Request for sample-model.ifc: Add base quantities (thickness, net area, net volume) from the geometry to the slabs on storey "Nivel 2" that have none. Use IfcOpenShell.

First a look at what the model holds.

```python
import ifcopenshell
import ifcopenshell.util.element
import ifcopenshell.util.unit

model = ifcopenshell.open("sample-model.ifc")
print(model.schema)
for unit_type in ("LENGTHUNIT", "AREAUNIT", "VOLUMEUNIT"):
    print(unit_type, ifcopenshell.util.unit.calculate_unit_scale(model, unit_type))
storey = next(s for s in model.by_type("IfcBuildingStorey") if s.Name == "Nivel 2")
slabs = [e for e in ifcopenshell.util.element.get_decomposition(storey) if e.is_a("IfcSlab")]
for e in sorted(slabs, key=lambda e: e.id()):
    print(e.id(), e.is_a(), e.Name, list(ifcopenshell.util.element.get_psets(e, qtos_only=True)), sep=" | ")
```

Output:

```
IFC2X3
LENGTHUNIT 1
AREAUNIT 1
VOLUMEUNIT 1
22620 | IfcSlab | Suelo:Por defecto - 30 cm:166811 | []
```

```python
import ifcopenshell
import ifcopenshell.api.pset
import ifcopenshell.geom
import ifcopenshell.util.element
import ifcopenshell.util.shape
import ifcopenshell.util.unit

model = ifcopenshell.open("sample-model.ifc")
unit_scale = ifcopenshell.util.unit.calculate_unit_scale(model)
area_scale = ifcopenshell.util.unit.calculate_unit_scale(model, "AREAUNIT")
volume_scale = ifcopenshell.util.unit.calculate_unit_scale(model, "VOLUMEUNIT")
settings = ifcopenshell.geom.settings()

storey = next(s for s in model.by_type("IfcBuildingStorey") if s.Name == "Nivel 2")
slabs = [e for e in ifcopenshell.util.element.get_decomposition(storey) if e.is_a("IfcSlab")]

for e in sorted(slabs, key=lambda e: e.id()):
    if ifcopenshell.util.element.get_psets(e, qtos_only=True, should_inherit=False):
        continue
    # Geometry comes back in metres, in the element's own axes.
    shape = ifcopenshell.geom.create_shape(settings, e)
    values = {
        "Width": ifcopenshell.util.shape.get_z(shape.geometry) / unit_scale,
        "NetArea": ifcopenshell.util.shape.get_footprint_area(shape.geometry) / area_scale,
        "NetVolume": ifcopenshell.util.shape.get_volume(shape.geometry) / volume_scale,
    }
    qto = ifcopenshell.api.pset.add_qto(model, product=e, name="BaseQuantities")
    ifcopenshell.api.pset.edit_qto(model, qto=qto, properties=values)
    print(e.id(), {k: round(v, 3) for k, v in values.items()})

model.write("sample-model_edited.ifc")
```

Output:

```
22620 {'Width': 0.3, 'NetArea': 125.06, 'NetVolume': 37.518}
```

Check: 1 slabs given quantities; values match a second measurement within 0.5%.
